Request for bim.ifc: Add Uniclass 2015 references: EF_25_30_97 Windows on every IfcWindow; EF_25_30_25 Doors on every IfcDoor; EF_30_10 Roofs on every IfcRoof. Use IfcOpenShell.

First a look at what the model holds.

```python
import ifcopenshell

model = ifcopenshell.open("bim.ifc")
print(model.schema)
print("classifications:", [c.Name for c in model.by_type("IfcClassification")])
for ifc_class in ("IfcDoor", "IfcRoof", "IfcStair", "IfcWall", "IfcWindow"):
    print(ifc_class, len(model.by_type(ifc_class)))
```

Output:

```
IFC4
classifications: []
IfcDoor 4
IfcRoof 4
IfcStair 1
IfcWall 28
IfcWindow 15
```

```python
import ifcopenshell
import ifcopenshell.api.classification

model = ifcopenshell.open("bim.ifc")

system = ifcopenshell.api.classification.add_classification(model, classification="Uniclass 2015")

codes = {
    "IfcWindow": ("EF_25_30_97", "Windows"),
    "IfcDoor": ("EF_25_30_25", "Doors"),
    "IfcRoof": ("EF_30_10", "Roofs"),
}
for ifc_class, (code, name) in codes.items():
    products = model.by_type(ifc_class)
    ifcopenshell.api.classification.add_reference(
        model, products=products, classification=system, identification=code, name=name
    )
    print(code, len(products))

model.write("bim-out.ifc")
```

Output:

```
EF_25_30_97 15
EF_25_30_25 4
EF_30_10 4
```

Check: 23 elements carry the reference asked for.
